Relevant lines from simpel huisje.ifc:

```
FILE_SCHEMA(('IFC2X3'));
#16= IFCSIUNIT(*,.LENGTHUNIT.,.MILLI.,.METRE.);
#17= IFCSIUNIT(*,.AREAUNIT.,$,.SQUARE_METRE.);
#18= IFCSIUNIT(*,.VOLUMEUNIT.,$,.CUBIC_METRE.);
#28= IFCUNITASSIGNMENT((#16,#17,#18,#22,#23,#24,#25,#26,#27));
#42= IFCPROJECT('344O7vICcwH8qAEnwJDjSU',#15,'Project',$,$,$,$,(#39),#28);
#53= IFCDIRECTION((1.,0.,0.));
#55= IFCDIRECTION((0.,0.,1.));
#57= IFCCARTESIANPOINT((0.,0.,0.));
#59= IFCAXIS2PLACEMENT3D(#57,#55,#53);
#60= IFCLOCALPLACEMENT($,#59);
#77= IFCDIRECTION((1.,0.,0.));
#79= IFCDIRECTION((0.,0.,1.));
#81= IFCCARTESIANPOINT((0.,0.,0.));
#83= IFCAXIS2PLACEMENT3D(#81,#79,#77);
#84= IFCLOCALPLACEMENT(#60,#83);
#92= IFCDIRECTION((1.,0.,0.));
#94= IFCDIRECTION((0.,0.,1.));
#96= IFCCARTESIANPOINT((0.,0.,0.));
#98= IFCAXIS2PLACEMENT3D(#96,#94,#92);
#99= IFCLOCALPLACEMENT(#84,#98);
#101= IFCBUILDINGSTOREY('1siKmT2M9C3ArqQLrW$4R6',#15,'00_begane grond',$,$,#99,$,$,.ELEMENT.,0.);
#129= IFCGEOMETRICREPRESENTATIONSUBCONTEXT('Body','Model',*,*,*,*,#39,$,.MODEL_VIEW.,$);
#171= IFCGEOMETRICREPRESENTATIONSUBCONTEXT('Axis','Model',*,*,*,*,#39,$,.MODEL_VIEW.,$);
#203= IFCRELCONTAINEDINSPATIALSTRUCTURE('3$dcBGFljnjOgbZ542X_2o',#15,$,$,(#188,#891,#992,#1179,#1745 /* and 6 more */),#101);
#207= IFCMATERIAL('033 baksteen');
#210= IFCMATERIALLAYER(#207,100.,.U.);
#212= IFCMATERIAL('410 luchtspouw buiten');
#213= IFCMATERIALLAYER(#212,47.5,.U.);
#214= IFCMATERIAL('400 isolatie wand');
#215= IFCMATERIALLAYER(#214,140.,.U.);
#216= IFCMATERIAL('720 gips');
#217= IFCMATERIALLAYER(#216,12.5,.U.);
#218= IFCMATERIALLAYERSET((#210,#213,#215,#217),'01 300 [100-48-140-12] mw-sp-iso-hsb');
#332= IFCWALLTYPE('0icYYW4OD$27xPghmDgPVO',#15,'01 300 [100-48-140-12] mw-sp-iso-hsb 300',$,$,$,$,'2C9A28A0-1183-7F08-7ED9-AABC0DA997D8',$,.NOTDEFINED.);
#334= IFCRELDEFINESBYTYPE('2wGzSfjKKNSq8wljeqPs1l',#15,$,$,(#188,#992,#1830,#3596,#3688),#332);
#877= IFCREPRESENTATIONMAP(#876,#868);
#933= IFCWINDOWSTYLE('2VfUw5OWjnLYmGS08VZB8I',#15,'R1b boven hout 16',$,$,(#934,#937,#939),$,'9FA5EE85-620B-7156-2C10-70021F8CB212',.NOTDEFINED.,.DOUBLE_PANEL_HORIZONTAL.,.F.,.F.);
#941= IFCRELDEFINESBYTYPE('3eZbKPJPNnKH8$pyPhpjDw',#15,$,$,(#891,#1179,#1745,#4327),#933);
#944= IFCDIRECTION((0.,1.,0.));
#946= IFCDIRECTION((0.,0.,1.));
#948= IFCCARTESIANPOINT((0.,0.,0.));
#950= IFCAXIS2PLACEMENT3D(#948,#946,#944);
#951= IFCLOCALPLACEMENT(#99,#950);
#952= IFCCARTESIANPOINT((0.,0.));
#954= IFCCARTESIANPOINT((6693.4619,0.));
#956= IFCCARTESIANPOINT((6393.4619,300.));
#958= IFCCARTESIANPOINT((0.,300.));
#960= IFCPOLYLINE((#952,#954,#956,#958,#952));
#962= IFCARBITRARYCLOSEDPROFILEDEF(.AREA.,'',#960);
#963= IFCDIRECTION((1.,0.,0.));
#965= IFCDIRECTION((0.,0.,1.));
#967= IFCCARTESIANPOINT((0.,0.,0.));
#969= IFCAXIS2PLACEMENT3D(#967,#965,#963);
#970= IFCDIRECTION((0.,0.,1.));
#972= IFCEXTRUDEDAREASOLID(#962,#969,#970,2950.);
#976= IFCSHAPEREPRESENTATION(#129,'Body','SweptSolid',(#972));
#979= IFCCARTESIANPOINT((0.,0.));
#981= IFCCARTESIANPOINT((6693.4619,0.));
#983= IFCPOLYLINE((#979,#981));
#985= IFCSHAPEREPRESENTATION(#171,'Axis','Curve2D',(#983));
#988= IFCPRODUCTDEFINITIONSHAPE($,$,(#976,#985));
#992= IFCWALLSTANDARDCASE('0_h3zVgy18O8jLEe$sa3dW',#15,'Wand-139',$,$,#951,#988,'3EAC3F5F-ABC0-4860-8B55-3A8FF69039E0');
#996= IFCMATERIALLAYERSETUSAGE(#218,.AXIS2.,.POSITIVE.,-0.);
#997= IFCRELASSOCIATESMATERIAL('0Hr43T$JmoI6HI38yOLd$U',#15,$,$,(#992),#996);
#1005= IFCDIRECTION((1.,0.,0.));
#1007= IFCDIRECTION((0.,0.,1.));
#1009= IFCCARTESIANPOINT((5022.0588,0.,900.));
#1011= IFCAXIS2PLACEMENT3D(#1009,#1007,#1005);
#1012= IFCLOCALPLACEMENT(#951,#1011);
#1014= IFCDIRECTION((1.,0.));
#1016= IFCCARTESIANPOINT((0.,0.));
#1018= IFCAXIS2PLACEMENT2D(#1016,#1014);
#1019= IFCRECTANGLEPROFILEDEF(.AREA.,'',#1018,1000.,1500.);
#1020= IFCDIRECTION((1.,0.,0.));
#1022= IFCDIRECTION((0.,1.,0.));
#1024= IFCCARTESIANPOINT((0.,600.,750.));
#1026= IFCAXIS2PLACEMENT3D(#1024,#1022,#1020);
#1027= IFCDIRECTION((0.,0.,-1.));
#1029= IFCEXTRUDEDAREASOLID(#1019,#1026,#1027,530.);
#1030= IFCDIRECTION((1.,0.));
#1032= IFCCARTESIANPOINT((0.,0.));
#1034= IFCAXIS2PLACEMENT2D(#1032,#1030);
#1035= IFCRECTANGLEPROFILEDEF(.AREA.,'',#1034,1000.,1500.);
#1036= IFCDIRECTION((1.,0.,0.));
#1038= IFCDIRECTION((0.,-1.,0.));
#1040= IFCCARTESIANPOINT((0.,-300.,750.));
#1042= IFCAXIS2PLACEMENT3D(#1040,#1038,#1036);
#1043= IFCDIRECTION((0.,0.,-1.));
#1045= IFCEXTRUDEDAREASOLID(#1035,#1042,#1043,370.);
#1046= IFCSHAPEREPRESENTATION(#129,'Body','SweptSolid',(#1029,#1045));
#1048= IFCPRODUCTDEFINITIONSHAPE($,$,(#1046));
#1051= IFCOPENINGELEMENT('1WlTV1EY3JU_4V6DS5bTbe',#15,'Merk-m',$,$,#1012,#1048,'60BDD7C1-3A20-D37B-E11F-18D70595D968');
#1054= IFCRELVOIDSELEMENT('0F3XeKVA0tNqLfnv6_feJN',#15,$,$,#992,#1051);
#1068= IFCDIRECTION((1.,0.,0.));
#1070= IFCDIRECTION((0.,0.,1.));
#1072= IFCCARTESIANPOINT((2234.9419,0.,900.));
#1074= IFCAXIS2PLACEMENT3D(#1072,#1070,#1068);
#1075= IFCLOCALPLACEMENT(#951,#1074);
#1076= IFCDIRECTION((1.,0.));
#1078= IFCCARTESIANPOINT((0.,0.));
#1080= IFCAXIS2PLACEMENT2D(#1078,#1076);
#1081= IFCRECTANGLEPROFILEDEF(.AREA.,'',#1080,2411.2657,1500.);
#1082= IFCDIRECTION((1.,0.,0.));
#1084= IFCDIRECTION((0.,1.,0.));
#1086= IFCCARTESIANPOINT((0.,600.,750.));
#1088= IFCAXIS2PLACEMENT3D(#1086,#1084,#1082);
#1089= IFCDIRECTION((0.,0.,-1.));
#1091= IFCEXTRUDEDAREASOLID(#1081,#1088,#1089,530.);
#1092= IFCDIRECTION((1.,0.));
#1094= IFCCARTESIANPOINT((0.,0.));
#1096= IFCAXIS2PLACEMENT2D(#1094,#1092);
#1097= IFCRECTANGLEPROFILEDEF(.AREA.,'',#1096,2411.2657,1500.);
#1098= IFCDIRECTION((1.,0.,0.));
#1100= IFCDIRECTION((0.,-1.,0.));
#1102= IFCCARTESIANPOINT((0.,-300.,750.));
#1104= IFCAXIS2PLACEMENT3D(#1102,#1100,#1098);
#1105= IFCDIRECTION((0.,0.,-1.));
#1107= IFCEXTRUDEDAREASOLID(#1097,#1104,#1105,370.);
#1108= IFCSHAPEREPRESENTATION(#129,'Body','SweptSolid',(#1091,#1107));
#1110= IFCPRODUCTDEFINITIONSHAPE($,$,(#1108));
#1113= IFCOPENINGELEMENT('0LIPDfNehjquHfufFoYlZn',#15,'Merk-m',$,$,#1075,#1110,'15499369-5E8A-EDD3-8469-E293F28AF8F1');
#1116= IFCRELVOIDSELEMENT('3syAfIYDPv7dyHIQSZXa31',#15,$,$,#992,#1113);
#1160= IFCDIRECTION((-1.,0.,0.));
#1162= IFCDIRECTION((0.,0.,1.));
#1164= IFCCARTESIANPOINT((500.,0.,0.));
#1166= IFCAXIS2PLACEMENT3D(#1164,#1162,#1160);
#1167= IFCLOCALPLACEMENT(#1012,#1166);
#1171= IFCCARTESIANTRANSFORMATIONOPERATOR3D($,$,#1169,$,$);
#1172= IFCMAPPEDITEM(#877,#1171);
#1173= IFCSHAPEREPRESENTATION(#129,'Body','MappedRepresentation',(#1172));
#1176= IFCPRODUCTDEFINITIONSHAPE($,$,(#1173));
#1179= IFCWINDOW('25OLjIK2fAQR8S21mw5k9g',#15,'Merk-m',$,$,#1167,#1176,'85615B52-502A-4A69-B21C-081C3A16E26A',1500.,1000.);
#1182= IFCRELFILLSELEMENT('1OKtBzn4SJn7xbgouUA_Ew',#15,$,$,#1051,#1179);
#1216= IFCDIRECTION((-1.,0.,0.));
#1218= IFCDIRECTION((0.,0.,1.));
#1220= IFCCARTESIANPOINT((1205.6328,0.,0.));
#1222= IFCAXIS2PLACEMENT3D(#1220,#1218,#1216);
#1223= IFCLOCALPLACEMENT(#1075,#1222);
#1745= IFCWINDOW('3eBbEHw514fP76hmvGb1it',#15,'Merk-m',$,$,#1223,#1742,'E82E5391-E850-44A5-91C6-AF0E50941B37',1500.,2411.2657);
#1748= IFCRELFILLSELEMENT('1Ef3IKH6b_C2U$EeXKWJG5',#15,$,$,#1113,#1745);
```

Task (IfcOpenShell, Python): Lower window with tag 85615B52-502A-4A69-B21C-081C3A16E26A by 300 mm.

```python
import numpy as np
import ifcopenshell
import ifcopenshell.api.geometry
import ifcopenshell.util.placement
import ifcopenshell.util.unit

model = ifcopenshell.open("simpel huisje.ifc")
unit_scale = ifcopenshell.util.unit.calculate_unit_scale(model)

window = model.by_id(1179)
opening = window.FillsVoids[0].RelatingOpeningElement
dz = -0.3 / unit_scale

shift = np.array([0.0, 0.0, dz])
# The window is placed relative to its opening, so it follows when the opening moves.
matrix = ifcopenshell.util.placement.get_local_placement(opening.ObjectPlacement)
matrix[:3, 3] += shift
ifcopenshell.api.geometry.edit_object_placement(
    model, product=opening, matrix=matrix, is_si=False, should_transform_children=True
)

print(f"moved by {dz * unit_scale:+.3f} m")

model.write("simpel huisje_v2.ifc")
```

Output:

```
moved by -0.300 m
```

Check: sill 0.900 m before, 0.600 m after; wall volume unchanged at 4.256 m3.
